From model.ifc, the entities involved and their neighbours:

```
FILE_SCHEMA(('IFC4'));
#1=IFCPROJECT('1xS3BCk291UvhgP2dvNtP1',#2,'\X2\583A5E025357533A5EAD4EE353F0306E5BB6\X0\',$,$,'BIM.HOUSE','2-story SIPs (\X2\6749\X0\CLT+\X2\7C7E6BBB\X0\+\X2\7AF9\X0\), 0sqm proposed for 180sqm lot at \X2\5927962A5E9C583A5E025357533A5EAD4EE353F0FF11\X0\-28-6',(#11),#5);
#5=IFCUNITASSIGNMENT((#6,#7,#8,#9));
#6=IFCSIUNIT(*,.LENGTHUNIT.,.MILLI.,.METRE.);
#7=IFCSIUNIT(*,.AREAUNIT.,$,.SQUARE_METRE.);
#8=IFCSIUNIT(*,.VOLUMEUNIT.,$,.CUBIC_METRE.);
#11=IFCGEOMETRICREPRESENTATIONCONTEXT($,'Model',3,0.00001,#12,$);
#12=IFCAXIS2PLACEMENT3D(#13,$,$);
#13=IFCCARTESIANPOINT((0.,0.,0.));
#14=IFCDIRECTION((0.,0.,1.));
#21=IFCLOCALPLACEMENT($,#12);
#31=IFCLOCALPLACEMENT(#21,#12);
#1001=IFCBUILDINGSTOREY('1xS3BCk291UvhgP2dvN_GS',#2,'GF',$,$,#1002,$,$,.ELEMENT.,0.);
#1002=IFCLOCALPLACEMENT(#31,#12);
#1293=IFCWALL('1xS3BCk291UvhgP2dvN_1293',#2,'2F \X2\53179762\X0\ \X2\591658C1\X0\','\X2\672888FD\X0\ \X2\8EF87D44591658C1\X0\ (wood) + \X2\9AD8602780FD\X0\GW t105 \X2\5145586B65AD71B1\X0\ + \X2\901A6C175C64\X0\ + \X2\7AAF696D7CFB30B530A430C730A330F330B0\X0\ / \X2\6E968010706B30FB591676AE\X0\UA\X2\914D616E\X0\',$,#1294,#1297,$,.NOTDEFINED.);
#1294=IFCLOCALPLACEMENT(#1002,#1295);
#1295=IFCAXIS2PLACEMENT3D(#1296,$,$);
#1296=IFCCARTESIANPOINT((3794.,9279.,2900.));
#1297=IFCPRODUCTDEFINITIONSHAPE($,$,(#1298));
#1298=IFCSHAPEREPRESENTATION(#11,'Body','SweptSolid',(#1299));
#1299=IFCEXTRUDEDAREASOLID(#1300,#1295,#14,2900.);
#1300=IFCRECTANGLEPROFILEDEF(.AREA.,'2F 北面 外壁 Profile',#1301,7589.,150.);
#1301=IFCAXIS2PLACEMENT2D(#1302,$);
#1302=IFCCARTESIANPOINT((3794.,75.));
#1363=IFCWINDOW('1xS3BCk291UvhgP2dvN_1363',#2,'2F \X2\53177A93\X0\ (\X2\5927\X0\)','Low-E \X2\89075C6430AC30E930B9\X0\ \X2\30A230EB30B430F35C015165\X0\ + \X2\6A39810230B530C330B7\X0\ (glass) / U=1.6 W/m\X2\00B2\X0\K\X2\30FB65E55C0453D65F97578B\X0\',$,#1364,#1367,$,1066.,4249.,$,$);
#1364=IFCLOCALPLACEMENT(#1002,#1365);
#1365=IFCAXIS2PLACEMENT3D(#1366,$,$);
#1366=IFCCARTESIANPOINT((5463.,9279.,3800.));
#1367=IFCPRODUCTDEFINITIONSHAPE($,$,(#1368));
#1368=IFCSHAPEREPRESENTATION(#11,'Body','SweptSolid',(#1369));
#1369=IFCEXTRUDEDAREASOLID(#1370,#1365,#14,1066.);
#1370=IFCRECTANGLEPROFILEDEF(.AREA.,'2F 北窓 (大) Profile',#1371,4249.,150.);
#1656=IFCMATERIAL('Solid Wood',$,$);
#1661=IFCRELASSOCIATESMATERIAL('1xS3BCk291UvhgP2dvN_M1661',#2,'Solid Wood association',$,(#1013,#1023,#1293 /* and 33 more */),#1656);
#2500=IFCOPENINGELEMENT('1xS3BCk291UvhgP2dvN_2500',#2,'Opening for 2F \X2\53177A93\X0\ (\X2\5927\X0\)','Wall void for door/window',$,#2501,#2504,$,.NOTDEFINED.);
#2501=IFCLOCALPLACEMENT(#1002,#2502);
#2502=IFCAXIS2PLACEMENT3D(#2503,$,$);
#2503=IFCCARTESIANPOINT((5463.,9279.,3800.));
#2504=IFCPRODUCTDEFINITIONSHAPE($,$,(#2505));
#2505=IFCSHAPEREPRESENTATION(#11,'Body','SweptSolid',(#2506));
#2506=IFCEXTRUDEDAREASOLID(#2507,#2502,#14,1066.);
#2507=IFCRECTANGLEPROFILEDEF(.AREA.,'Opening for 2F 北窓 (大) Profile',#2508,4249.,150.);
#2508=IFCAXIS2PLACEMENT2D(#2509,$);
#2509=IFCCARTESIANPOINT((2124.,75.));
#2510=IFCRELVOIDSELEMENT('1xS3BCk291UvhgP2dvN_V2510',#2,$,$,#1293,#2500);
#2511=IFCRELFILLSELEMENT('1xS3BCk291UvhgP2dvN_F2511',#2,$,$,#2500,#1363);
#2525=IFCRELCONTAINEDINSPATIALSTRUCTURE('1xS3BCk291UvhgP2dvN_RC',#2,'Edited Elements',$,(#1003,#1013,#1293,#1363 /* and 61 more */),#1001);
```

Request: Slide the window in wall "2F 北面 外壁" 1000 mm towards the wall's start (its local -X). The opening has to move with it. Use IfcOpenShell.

```python
import ifcopenshell
import ifcopenshell.api.geometry
import ifcopenshell.util.placement
import ifcopenshell.util.unit

model = ifcopenshell.open("model.ifc")
unit_scale = ifcopenshell.util.unit.calculate_unit_scale(model)

window = model.by_id(1363)
opening = window.FillsVoids[0].RelatingOpeningElement
wall = opening.VoidsElements[0].RelatingBuildingElement

wall_matrix = ifcopenshell.util.placement.get_local_placement(wall.ObjectPlacement)
shift = wall_matrix[:3, 0] * -1 / unit_scale
before = ifcopenshell.util.placement.get_local_placement(window.ObjectPlacement)[:3, 3].copy()

# The window is not placed relative to its opening, so move both.
for product in (opening, window):
    matrix = ifcopenshell.util.placement.get_local_placement(product.ObjectPlacement)
    matrix[:3, 3] += shift
    ifcopenshell.api.geometry.edit_object_placement(model, product=product, matrix=matrix, is_si=False)

after = ifcopenshell.util.placement.get_local_placement(window.ObjectPlacement)[:3, 3]
print("window moved by", (after - before).round(3) + 0.0)

model.write("model_updated.ifc")
```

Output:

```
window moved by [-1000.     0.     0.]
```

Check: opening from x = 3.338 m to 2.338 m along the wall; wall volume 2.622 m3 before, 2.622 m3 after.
